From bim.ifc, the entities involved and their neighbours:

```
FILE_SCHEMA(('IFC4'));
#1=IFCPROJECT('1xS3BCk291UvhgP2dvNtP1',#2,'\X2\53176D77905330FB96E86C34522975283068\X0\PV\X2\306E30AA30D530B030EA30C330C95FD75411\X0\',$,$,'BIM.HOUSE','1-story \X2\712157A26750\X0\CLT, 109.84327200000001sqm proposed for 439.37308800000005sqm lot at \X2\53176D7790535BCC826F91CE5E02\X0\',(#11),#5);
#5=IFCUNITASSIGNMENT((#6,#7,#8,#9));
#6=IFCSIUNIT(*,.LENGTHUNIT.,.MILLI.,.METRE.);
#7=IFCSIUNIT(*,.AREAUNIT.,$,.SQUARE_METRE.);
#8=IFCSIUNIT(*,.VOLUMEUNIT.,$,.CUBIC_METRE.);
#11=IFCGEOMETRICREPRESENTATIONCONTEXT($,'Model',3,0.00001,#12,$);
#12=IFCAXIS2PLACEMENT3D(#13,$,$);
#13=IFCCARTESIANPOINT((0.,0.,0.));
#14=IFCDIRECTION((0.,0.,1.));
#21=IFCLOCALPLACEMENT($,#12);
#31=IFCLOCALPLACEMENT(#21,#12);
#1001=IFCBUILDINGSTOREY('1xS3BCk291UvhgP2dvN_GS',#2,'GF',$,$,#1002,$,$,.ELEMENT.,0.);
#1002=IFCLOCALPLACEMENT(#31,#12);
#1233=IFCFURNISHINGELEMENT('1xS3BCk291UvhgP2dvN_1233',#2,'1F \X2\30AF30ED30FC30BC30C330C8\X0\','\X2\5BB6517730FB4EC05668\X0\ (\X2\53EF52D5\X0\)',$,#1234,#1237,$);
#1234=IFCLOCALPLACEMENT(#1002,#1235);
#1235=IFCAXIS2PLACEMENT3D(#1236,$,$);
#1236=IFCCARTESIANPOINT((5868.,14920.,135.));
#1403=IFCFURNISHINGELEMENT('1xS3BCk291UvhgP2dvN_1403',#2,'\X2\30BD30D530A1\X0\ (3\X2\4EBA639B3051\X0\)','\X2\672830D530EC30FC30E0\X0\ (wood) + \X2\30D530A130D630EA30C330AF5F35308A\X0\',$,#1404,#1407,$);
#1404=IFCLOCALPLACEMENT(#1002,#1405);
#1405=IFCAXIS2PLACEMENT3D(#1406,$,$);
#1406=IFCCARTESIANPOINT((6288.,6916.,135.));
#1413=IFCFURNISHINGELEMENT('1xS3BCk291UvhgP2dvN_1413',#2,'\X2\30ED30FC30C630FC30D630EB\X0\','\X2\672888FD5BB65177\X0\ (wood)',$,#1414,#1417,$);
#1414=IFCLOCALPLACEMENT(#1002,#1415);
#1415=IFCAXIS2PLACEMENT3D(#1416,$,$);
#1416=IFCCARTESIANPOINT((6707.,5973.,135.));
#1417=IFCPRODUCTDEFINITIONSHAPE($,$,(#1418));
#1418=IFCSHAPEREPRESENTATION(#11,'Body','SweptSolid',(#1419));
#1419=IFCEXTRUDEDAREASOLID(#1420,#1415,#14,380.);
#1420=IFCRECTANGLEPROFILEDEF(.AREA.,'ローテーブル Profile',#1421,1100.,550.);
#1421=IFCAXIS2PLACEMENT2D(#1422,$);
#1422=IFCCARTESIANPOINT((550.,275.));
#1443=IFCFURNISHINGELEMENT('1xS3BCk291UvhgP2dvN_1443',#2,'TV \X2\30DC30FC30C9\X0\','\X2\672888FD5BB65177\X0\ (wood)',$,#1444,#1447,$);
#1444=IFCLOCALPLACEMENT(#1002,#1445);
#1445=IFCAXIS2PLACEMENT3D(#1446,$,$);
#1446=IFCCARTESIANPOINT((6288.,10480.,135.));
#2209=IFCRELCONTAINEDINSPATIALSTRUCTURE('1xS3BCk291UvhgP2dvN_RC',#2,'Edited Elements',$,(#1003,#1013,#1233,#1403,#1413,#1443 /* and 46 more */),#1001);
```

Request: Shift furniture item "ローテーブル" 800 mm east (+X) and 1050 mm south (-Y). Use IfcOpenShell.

```python
import ifcopenshell
import ifcopenshell.api.geometry
import ifcopenshell.util.placement
import ifcopenshell.util.unit

model = ifcopenshell.open("bim.ifc")
unit_scale = ifcopenshell.util.unit.calculate_unit_scale(model)

item = model.by_id(1413)
matrix = ifcopenshell.util.placement.get_local_placement(item.ObjectPlacement)
matrix[0, 3] += 0.8 / unit_scale
matrix[1, 3] -= 1.05 / unit_scale
ifcopenshell.api.geometry.edit_object_placement(model, product=item, matrix=matrix, is_si=False)

print(ifcopenshell.util.placement.get_local_placement(item.ObjectPlacement).round(3) + 0.0)

model.write("bim_v2.ifc")
```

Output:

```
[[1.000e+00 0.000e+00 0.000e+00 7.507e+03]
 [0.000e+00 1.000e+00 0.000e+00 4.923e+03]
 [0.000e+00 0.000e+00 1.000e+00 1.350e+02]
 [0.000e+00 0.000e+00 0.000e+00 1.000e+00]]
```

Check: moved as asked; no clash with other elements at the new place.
